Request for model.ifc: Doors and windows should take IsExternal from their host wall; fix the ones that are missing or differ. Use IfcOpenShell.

First a look at what the model holds.

```python
import ifcopenshell
import ifcopenshell.util.element

model = ifcopenshell.open("model.ifc")
print(model.schema)
seen = {}
for e in model.by_type("IfcDoor") + model.by_type("IfcWindow"):
    if not e.FillsVoids:
        continue
    host = e.FillsVoids[0].RelatingOpeningElement.VoidsElements[0].RelatingBuildingElement
    own = ifcopenshell.util.element.get_pset(e, f"Pset_{e.is_a()[3:].removesuffix('StandardCase')}Common", "IsExternal")
    wall = ifcopenshell.util.element.get_pset(host, "Pset_WallCommon", "IsExternal")
    seen[e.is_a(), own, wall] = seen.get((e.is_a(), own, wall), 0) + 1
for (cls, own, wall), count in sorted(seen.items(), key=str):
    print(count, cls, "IsExternal:", own, "| host wall:", wall)
```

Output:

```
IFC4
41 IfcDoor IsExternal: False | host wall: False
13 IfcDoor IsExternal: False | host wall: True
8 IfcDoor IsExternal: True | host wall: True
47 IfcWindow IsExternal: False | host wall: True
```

```python
import ifcopenshell
import ifcopenshell.api.pset
import ifcopenshell.util.element

model = ifcopenshell.open("model.ifc")

count = 0
for ifc_class, pset_name in (("IfcDoor", "Pset_DoorCommon"), ("IfcWindow", "Pset_WindowCommon")):
    for e in model.by_type(ifc_class):
        if not e.FillsVoids:
            continue
        host = e.FillsVoids[0].RelatingOpeningElement.VoidsElements[0].RelatingBuildingElement
        external = ifcopenshell.util.element.get_pset(host, "Pset_WallCommon", "IsExternal")
        if external is None or ifcopenshell.util.element.get_pset(e, pset_name, "IsExternal") == external:
            continue
        pset = ifcopenshell.api.pset.add_pset(model, product=e, name=pset_name)
        ifcopenshell.api.pset.edit_pset(model, pset=pset, properties={"IsExternal": external})
        count += 1

print(count, "updated")

model.write("model_edited.ifc")
```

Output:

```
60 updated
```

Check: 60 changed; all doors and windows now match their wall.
